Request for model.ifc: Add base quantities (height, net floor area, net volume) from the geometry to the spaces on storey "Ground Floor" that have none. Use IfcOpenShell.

First a look at what the model holds.

```python
import ifcopenshell
import ifcopenshell.util.element
import ifcopenshell.util.unit

model = ifcopenshell.open("model.ifc")
print(model.schema)
for unit_type in ("LENGTHUNIT", "AREAUNIT", "VOLUMEUNIT"):
    print(unit_type, ifcopenshell.util.unit.calculate_unit_scale(model, unit_type))
storey = next(s for s in model.by_type("IfcBuildingStorey") if s.Name == "Ground Floor")
spaces = [e for e in ifcopenshell.util.element.get_decomposition(storey) if e.is_a("IfcSpace")]
for e in sorted(spaces, key=lambda e: e.id()):
    print(e.id(), e.is_a(), e.Name, list(ifcopenshell.util.element.get_psets(e, qtos_only=True)), sep=" | ")
```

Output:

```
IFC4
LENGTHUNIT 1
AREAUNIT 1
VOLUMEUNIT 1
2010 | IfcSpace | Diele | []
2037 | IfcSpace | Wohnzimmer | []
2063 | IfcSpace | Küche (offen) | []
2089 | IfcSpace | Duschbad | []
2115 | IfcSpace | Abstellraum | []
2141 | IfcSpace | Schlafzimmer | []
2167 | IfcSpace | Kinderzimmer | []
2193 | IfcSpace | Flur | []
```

```python
import ifcopenshell
import ifcopenshell.api.pset
import ifcopenshell.geom
import ifcopenshell.util.element
import ifcopenshell.util.shape
import ifcopenshell.util.unit

model = ifcopenshell.open("model.ifc")
unit_scale = ifcopenshell.util.unit.calculate_unit_scale(model)
area_scale = ifcopenshell.util.unit.calculate_unit_scale(model, "AREAUNIT")
volume_scale = ifcopenshell.util.unit.calculate_unit_scale(model, "VOLUMEUNIT")
settings = ifcopenshell.geom.settings()

storey = next(s for s in model.by_type("IfcBuildingStorey") if s.Name == "Ground Floor")
spaces = [e for e in ifcopenshell.util.element.get_decomposition(storey) if e.is_a("IfcSpace")]

for e in sorted(spaces, key=lambda e: e.id()):
    if ifcopenshell.util.element.get_psets(e, qtos_only=True, should_inherit=False):
        continue
    # Geometry comes back in metres, in the element's own axes.
    shape = ifcopenshell.geom.create_shape(settings, e)
    values = {
        "Height": ifcopenshell.util.shape.get_z(shape.geometry) / unit_scale,
        "NetFloorArea": ifcopenshell.util.shape.get_footprint_area(shape.geometry) / area_scale,
        "NetVolume": ifcopenshell.util.shape.get_volume(shape.geometry) / volume_scale,
    }
    qto = ifcopenshell.api.pset.add_qto(model, product=e, name="Qto_SpaceBaseQuantities")
    ifcopenshell.api.pset.edit_qto(model, qto=qto, properties=values)
    print(e.id(), {k: round(v, 3) for k, v in values.items()})

model.write("model_updated.ifc")
```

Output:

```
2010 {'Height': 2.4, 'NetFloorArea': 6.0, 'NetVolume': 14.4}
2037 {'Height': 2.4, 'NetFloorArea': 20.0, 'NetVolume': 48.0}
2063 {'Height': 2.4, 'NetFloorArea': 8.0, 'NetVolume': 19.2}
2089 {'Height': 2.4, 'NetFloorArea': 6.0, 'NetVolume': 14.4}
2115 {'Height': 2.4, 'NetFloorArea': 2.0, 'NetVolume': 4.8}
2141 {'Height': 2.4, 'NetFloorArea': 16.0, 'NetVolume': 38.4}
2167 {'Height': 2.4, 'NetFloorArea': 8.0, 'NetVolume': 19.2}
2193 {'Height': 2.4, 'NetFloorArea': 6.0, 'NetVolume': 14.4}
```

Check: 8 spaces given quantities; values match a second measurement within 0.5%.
